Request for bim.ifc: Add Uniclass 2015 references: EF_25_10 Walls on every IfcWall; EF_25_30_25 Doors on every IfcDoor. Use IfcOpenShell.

First a look at what the model holds.

```python
import ifcopenshell

model = ifcopenshell.open("bim.ifc")
print(model.schema)
print("classifications:", [c.Name for c in model.by_type("IfcClassification")])
for ifc_class in ("IfcDoor", "IfcRoof", "IfcStair", "IfcWall", "IfcWindow"):
    print(ifc_class, len(model.by_type(ifc_class)))
```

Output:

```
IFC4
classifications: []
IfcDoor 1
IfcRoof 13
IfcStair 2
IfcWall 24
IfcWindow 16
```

```python
import ifcopenshell
import ifcopenshell.api.classification

model = ifcopenshell.open("bim.ifc")

system = ifcopenshell.api.classification.add_classification(model, classification="Uniclass 2015")

codes = {
    "IfcWall": ("EF_25_10", "Walls"),
    "IfcDoor": ("EF_25_30_25", "Doors"),
}
for ifc_class, (code, name) in codes.items():
    products = model.by_type(ifc_class)
    ifcopenshell.api.classification.add_reference(
        model, products=products, classification=system, identification=code, name=name
    )
    print(code, len(products))

model.write("bim-out.ifc")
```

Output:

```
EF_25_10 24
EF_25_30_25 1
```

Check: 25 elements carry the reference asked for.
